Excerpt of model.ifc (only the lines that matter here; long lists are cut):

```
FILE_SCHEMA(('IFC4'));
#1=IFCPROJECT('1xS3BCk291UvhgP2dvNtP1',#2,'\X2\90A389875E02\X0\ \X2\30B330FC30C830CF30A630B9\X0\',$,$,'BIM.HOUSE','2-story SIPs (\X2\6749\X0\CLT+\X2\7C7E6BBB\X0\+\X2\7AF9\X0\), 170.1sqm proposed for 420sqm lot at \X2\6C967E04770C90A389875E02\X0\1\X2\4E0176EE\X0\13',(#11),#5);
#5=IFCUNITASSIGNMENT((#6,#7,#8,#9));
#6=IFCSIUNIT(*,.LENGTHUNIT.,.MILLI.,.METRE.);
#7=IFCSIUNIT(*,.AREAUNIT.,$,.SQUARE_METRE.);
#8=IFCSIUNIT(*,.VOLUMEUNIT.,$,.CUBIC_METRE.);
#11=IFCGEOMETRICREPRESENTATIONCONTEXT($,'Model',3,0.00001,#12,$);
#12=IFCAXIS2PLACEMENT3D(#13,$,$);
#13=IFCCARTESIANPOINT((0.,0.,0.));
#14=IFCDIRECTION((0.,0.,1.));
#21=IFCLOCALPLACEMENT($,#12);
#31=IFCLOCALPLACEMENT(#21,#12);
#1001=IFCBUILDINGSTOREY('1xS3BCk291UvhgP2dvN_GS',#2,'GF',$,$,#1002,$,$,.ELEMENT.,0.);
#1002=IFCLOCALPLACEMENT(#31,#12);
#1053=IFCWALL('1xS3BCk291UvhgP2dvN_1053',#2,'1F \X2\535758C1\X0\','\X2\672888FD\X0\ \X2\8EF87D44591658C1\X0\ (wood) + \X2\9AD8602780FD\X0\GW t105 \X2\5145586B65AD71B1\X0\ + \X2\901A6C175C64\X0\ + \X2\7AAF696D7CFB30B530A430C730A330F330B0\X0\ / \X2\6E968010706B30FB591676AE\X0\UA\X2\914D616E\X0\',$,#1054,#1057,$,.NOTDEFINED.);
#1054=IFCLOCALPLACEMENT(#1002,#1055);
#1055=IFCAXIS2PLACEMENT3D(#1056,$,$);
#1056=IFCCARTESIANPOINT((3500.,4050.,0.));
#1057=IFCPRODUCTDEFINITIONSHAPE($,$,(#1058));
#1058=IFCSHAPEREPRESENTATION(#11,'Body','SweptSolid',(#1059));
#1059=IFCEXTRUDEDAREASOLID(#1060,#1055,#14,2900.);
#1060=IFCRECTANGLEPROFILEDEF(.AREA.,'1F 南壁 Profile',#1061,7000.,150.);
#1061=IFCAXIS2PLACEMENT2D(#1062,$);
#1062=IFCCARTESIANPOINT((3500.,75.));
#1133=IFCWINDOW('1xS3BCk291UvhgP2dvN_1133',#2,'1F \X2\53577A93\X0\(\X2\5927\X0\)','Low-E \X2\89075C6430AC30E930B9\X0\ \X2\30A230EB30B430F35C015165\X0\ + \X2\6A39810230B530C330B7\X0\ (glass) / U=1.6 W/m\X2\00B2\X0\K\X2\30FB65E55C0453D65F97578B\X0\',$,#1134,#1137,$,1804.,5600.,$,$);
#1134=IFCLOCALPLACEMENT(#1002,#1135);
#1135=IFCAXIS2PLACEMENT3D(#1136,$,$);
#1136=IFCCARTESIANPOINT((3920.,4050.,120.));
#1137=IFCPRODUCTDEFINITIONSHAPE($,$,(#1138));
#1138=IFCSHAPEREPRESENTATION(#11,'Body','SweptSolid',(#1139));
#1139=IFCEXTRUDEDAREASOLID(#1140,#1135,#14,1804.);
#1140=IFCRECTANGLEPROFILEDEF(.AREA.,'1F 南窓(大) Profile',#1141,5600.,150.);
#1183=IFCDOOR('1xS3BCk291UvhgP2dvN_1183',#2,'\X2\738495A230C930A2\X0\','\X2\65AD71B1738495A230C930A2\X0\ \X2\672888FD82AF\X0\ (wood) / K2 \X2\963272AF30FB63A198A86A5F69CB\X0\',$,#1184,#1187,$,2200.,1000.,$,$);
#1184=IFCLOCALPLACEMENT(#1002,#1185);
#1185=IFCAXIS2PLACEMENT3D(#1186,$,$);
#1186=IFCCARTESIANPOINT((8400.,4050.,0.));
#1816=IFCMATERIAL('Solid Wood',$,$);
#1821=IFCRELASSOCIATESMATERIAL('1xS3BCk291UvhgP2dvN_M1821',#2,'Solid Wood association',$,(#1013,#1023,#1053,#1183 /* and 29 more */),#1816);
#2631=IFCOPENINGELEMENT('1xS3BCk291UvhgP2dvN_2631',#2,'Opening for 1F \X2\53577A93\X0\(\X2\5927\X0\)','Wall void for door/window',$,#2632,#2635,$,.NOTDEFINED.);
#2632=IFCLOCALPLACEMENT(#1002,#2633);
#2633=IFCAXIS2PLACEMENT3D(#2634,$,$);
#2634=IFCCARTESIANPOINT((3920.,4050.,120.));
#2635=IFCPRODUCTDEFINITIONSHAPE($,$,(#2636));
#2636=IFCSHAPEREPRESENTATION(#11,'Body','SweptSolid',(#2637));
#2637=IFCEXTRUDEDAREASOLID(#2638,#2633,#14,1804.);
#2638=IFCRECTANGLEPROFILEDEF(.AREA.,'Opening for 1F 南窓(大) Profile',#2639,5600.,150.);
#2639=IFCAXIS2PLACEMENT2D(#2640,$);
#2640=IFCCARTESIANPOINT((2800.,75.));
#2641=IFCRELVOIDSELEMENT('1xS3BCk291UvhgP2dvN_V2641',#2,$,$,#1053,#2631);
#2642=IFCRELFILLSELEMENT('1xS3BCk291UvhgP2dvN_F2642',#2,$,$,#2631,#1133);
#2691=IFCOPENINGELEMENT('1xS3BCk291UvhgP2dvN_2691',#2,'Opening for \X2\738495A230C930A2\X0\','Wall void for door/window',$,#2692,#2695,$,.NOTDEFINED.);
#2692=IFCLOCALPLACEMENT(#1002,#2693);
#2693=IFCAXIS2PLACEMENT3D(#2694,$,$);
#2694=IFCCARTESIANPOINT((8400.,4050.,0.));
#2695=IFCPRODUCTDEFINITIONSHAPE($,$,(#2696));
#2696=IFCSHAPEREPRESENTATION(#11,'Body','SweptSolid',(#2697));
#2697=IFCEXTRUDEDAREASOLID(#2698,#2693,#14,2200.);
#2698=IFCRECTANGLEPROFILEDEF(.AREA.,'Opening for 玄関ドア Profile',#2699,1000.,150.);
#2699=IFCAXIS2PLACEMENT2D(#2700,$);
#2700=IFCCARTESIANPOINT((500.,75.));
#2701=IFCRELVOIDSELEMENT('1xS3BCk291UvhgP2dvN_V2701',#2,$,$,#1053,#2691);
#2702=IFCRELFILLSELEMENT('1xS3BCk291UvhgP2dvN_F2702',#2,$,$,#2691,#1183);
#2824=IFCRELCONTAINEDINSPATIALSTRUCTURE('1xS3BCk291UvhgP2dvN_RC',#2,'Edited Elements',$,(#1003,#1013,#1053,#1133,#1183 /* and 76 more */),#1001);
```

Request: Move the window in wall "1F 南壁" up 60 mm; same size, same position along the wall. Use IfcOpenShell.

```python
import numpy as np
import ifcopenshell
import ifcopenshell.api.geometry
import ifcopenshell.util.placement
import ifcopenshell.util.unit

model = ifcopenshell.open("model.ifc")
unit_scale = ifcopenshell.util.unit.calculate_unit_scale(model)

window = model.by_guid("1xS3BCk291UvhgP2dvN_1133")
opening = window.FillsVoids[0].RelatingOpeningElement
dz = 60.0

shift = np.array([0.0, 0.0, dz])
# The window is not placed relative to its opening, so move both.
for product in (opening, window):
    matrix = ifcopenshell.util.placement.get_local_placement(product.ObjectPlacement)
    matrix[:3, 3] += shift
    ifcopenshell.api.geometry.edit_object_placement(model, product=product, matrix=matrix, is_si=False)

print(f"moved by {dz * unit_scale:+.3f} m")

model.write("model-out.ifc")
```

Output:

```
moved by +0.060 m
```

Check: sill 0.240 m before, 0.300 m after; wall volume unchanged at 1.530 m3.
